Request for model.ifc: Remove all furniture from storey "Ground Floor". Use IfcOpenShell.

First a look at what the model holds.

```python
import ifcopenshell
import ifcopenshell.util.element

model = ifcopenshell.open("model.ifc")
print(model.schema)
storey = next(s for s in model.by_type("IfcBuildingStorey") if s.Name == "Ground Floor")
furniture = [e for e in ifcopenshell.util.element.get_decomposition(storey) if e.is_a("IfcFurnishingElement")]
seen = {}
for e in furniture:
    element_type = ifcopenshell.util.element.get_type(e)
    name = element_type.Name if element_type not in (None, e) else None
    seen[name] = seen.get(name, 0) + 1
for name, count in sorted(seen.items(), key=str):
    print(count, "x", name)
```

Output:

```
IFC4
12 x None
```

```python
import ifcopenshell
import ifcopenshell.api.root
import ifcopenshell.util.element

model = ifcopenshell.open("model.ifc")

storey = next(s for s in model.by_type("IfcBuildingStorey") if s.Name == "Ground Floor")
furniture = [e for e in ifcopenshell.util.element.get_decomposition(storey) if e.is_a("IfcFurnishingElement")]

for e in furniture:
    ifcopenshell.api.root.remove_product(model, product=e)
print(len(furniture), "removed")

model.write("model_rev.ifc")
```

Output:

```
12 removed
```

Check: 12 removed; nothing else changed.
